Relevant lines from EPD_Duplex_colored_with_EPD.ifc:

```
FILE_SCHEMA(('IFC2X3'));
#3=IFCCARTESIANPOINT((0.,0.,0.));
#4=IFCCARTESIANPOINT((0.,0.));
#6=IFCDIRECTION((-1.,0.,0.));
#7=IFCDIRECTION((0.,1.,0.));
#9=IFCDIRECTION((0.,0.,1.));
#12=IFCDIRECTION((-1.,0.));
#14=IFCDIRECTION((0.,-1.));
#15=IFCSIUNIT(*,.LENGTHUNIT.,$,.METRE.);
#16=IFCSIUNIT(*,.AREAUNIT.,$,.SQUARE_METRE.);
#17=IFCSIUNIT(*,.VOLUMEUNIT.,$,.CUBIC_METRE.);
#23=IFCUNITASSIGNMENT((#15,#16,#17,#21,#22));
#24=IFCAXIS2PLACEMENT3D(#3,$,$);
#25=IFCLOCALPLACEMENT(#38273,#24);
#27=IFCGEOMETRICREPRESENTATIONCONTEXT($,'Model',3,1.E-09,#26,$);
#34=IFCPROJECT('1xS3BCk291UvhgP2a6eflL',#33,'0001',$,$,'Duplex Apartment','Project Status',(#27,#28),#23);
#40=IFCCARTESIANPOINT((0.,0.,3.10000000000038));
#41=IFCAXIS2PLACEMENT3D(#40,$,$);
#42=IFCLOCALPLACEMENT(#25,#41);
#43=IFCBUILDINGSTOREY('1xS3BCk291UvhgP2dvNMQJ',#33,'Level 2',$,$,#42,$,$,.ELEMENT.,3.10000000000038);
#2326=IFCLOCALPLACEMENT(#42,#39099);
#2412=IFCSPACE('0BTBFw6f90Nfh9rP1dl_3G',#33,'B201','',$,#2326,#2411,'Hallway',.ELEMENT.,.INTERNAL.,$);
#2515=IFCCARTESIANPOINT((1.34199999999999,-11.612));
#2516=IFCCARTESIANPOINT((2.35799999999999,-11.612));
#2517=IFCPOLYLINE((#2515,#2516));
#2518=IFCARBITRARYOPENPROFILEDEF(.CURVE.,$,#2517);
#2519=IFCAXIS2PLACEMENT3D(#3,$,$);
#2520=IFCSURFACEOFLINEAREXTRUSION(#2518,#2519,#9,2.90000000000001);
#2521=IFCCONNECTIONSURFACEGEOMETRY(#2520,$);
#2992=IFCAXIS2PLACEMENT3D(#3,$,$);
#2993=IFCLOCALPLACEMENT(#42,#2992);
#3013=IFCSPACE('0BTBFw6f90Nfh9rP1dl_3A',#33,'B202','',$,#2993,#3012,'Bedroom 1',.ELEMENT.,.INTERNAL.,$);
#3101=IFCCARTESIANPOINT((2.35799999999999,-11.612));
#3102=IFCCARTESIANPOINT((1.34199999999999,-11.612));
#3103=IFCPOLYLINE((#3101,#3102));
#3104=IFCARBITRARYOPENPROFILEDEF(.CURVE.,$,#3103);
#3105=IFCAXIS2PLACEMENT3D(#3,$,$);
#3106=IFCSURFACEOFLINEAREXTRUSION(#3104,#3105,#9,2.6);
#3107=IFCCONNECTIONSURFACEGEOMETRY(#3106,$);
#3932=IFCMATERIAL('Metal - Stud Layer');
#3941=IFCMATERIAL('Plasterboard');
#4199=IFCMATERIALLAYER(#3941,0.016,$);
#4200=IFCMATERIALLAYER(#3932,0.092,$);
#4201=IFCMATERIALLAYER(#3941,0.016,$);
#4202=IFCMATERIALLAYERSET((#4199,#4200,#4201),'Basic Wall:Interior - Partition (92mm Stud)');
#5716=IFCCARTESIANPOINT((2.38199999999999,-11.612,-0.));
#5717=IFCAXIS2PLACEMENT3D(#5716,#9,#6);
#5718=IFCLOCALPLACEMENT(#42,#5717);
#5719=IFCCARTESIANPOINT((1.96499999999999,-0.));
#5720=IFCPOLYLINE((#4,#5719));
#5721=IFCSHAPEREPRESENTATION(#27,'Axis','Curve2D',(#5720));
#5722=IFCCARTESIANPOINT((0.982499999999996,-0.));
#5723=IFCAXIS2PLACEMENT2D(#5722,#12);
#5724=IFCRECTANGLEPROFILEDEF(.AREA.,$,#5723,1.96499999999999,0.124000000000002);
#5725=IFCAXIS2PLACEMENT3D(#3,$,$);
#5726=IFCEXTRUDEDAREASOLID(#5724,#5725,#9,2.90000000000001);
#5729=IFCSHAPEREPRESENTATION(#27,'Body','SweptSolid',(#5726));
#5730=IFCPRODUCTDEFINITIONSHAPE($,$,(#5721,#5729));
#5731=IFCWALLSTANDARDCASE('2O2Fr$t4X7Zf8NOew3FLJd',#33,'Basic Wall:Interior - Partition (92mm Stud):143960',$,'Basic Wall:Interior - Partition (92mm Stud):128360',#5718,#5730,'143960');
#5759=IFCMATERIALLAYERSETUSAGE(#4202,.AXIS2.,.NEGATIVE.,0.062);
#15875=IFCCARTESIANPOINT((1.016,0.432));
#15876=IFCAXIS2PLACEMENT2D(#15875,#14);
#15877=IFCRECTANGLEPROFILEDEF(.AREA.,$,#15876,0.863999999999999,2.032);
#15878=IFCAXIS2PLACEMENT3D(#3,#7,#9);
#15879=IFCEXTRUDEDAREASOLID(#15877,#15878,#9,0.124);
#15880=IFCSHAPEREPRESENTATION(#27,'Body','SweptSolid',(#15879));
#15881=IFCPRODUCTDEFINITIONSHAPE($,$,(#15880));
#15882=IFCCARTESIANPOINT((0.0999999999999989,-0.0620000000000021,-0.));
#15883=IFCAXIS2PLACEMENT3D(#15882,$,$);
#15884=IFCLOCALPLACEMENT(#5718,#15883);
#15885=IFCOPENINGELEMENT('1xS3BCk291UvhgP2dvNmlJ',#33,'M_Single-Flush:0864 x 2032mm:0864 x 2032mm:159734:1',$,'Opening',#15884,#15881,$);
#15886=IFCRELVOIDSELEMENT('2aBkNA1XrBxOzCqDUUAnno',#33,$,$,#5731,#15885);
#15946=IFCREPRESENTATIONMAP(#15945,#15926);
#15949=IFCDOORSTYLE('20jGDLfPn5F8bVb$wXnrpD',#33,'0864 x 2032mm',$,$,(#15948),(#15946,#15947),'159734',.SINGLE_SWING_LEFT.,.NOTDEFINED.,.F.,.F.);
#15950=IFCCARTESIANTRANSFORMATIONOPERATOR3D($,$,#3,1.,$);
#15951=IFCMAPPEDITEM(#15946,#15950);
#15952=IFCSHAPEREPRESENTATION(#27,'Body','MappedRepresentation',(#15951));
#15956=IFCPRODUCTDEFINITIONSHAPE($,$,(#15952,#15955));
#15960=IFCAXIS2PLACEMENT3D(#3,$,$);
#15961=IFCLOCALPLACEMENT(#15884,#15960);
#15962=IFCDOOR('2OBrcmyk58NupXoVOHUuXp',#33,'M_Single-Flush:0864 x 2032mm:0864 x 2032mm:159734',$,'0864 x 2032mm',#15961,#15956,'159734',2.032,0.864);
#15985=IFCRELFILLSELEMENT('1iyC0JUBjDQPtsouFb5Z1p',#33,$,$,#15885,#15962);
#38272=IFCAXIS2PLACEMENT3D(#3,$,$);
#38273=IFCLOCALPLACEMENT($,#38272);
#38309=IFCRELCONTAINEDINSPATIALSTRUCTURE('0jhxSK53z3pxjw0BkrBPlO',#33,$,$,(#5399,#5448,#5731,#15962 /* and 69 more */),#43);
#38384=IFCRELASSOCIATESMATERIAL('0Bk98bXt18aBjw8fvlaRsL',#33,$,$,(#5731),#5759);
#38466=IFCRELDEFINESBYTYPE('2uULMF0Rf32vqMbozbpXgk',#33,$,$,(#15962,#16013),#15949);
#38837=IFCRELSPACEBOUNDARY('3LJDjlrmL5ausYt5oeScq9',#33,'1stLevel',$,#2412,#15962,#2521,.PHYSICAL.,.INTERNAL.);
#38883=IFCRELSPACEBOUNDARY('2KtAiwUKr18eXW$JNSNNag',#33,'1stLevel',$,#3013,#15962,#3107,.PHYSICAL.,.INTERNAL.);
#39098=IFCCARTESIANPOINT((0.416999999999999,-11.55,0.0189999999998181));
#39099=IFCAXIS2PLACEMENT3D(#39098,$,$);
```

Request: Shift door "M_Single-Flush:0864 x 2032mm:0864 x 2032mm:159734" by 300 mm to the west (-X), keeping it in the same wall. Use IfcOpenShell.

```python
import numpy as np
import ifcopenshell
import ifcopenshell.api.geometry
import ifcopenshell.util.placement
import ifcopenshell.util.unit

model = ifcopenshell.open("EPD_Duplex_colored_with_EPD.ifc")
unit_scale = ifcopenshell.util.unit.calculate_unit_scale(model)

door = model.by_id(15962)
opening = door.FillsVoids[0].RelatingOpeningElement
wall = opening.VoidsElements[0].RelatingBuildingElement

wall_matrix = ifcopenshell.util.placement.get_local_placement(wall.ObjectPlacement)
shift = wall_matrix[:3, 0] * 0.3 / unit_scale
before = ifcopenshell.util.placement.get_local_placement(door.ObjectPlacement)[:3, 3].copy()

# The door is placed relative to its opening, so it follows when the opening moves.
matrix = ifcopenshell.util.placement.get_local_placement(opening.ObjectPlacement)
matrix[:3, 3] += shift
ifcopenshell.api.geometry.edit_object_placement(
    model, product=opening, matrix=matrix, is_si=False, should_transform_children=True
)

# Space boundary surfaces are stored in each space's coordinates; move them too.
for rel in door.ProvidesBoundaries:
    if not rel.ConnectionGeometry:
        continue
    surface = rel.ConnectionGeometry.SurfaceOnRelatingElement
    space_matrix = ifcopenshell.util.placement.get_local_placement(rel.RelatingSpace.ObjectPlacement)
    point = np.array(surface.Position.Location.Coordinates) + space_matrix[:3, :3].T @ shift
    surface.Position = model.createIfcAxis2Placement3D(
        model.createIfcCartesianPoint(point.tolist()), surface.Position.Axis, surface.Position.RefDirection
    )

after = ifcopenshell.util.placement.get_local_placement(door.ObjectPlacement)[:3, 3]
print("door moved by", (after - before).round(3) + 0.0)

model.write("EPD_Duplex_colored_with_EPD_rev.ifc")
```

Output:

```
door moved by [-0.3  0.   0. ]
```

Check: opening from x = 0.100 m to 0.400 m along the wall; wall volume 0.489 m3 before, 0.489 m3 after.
